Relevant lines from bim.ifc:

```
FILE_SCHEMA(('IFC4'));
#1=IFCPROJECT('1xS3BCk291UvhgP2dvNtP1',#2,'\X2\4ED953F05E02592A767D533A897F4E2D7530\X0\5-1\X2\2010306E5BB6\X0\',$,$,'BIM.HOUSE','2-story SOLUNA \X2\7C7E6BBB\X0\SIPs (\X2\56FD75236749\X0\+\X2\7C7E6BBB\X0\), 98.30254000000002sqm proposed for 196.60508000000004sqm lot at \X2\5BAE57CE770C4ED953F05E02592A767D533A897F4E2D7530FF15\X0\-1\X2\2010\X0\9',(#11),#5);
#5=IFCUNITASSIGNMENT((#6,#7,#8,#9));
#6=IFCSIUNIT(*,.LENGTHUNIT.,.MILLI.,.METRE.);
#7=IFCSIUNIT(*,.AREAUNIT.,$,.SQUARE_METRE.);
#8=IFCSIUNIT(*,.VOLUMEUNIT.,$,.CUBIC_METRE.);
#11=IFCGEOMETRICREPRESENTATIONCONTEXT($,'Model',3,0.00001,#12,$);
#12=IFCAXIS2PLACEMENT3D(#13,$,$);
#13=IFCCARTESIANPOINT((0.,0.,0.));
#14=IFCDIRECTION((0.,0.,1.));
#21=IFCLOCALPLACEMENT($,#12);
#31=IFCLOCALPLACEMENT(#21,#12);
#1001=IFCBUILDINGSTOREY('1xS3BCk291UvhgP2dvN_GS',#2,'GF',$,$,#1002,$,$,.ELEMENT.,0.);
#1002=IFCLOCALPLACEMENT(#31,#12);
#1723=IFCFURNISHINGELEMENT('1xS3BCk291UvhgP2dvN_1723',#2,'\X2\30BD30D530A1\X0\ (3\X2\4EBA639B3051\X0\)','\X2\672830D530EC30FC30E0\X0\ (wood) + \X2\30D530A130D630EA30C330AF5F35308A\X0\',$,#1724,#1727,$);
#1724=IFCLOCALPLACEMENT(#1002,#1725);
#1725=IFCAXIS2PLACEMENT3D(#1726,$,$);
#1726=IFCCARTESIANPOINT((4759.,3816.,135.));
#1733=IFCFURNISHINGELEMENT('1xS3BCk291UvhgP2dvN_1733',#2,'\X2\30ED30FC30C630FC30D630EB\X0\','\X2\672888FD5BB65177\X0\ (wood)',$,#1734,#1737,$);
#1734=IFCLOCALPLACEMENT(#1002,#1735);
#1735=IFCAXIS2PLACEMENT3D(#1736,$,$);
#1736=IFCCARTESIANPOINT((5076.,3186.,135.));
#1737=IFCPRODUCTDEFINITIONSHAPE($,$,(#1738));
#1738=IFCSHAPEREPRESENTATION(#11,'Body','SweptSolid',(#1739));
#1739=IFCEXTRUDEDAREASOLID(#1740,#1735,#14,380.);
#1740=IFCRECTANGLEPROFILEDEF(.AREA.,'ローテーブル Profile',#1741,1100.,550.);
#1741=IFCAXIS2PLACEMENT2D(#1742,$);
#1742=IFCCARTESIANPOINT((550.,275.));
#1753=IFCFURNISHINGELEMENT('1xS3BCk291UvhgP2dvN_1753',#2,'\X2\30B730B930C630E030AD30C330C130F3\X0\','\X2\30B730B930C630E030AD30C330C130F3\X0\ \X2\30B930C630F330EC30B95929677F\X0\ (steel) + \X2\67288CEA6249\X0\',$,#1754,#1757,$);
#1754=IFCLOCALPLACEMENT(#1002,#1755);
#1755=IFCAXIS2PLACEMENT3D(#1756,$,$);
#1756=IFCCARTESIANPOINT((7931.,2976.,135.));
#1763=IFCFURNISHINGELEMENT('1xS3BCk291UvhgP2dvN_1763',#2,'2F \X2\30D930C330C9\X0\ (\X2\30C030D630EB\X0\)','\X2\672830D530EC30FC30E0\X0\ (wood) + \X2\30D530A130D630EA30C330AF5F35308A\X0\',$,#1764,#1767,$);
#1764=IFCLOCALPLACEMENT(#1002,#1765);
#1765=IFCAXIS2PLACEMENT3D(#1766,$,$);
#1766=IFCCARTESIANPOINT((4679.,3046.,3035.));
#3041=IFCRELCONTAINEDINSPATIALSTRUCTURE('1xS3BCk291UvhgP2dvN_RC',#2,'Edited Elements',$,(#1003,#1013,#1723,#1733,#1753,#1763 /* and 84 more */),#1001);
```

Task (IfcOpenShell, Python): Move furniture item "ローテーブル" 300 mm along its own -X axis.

```python
import ifcopenshell
import ifcopenshell.api.geometry
import ifcopenshell.util.placement

model = ifcopenshell.open("bim.ifc")

item = model.by_guid("1xS3BCk291UvhgP2dvN_1733")
matrix = ifcopenshell.util.placement.get_local_placement(item.ObjectPlacement)
matrix[:3, 3] -= matrix[:3, 0] * 300.0
ifcopenshell.api.geometry.edit_object_placement(model, product=item, matrix=matrix, is_si=False)

print(ifcopenshell.util.placement.get_local_placement(item.ObjectPlacement).round(3) + 0.0)

model.write("bim-out.ifc")
```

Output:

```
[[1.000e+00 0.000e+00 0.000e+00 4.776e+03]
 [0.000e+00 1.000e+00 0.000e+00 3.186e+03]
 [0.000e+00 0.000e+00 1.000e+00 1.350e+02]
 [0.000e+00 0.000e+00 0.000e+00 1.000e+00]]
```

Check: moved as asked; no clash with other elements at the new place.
